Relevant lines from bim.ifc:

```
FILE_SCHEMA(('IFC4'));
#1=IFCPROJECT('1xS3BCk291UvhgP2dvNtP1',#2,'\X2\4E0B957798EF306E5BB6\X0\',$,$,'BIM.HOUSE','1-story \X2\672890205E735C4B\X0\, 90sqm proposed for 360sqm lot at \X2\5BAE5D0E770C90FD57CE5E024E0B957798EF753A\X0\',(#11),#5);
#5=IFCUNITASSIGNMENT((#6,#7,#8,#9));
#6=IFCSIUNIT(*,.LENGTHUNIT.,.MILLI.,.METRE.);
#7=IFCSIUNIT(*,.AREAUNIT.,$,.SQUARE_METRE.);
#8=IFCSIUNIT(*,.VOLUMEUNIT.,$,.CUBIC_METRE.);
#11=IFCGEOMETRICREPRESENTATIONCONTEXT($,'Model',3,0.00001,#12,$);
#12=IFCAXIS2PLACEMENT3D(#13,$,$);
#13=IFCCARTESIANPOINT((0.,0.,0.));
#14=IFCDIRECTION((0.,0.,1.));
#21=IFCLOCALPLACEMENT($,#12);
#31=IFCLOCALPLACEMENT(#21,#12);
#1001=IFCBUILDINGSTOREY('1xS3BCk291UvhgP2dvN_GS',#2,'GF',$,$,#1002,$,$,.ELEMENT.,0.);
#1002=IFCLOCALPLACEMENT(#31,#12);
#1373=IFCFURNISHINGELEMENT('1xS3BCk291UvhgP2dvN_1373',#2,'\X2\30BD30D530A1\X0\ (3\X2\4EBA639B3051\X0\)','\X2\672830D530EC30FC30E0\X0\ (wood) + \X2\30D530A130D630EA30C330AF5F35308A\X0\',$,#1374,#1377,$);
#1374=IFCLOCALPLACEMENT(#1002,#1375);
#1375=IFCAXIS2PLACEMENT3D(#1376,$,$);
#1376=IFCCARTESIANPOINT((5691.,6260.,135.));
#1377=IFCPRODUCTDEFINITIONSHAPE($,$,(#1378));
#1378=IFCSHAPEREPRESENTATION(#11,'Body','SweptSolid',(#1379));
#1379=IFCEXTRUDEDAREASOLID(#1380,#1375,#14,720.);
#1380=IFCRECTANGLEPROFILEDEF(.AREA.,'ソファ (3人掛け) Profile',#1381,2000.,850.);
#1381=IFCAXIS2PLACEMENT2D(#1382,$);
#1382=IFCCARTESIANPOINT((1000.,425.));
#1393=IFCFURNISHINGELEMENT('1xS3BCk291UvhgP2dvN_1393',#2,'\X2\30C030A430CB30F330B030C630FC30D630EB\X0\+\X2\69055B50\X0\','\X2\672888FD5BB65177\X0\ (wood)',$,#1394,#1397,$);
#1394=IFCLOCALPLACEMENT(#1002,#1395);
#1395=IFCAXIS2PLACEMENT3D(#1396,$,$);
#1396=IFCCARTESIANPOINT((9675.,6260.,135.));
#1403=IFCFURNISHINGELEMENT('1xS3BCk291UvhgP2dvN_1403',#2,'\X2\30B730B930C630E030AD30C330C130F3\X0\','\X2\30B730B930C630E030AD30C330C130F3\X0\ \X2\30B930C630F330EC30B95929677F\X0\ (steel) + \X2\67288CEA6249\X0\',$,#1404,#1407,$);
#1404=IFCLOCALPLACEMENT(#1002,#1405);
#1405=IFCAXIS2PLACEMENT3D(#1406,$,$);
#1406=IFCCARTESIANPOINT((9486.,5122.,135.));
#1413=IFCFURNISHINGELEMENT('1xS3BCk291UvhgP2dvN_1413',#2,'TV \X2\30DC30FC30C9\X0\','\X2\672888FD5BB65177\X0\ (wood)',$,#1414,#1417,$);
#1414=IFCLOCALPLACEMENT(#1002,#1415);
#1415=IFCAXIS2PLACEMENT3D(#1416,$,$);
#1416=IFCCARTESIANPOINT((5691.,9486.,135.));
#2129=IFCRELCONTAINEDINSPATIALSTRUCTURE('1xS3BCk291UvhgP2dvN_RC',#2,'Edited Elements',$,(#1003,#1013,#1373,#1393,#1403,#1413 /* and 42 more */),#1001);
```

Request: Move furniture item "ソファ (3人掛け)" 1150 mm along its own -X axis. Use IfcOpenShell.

```python
import ifcopenshell
import ifcopenshell.api.geometry
import ifcopenshell.util.placement
import ifcopenshell.util.unit

model = ifcopenshell.open("bim.ifc")
unit_scale = ifcopenshell.util.unit.calculate_unit_scale(model)

item = model.by_guid("1xS3BCk291UvhgP2dvN_1373")
matrix = ifcopenshell.util.placement.get_local_placement(item.ObjectPlacement)
matrix[:3, 3] -= matrix[:3, 0] * 1.15 / unit_scale
ifcopenshell.api.geometry.edit_object_placement(model, product=item, matrix=matrix, is_si=False)

print(ifcopenshell.util.placement.get_local_placement(item.ObjectPlacement).round(3) + 0.0)

model.write("bim_v2.ifc")
```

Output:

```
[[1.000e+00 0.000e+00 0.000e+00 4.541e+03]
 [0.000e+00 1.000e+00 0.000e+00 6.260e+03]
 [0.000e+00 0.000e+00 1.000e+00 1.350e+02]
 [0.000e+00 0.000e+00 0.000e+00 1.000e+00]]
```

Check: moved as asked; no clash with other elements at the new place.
